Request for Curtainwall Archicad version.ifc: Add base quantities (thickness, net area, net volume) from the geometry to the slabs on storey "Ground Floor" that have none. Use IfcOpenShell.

First a look at what the model holds.

```python
import ifcopenshell
import ifcopenshell.util.element
import ifcopenshell.util.unit

model = ifcopenshell.open("Curtainwall Archicad version.ifc")
print(model.schema)
for unit_type in ("LENGTHUNIT", "AREAUNIT", "VOLUMEUNIT"):
    print(unit_type, ifcopenshell.util.unit.calculate_unit_scale(model, unit_type))
storey = next(s for s in model.by_type("IfcBuildingStorey") if s.Name == "Ground Floor")
slabs = [e for e in ifcopenshell.util.element.get_decomposition(storey) if e.is_a("IfcSlab")]
for e in sorted(slabs, key=lambda e: e.id()):
    print(e.id(), e.is_a(), e.Name, list(ifcopenshell.util.element.get_psets(e, qtos_only=True)), sep=" | ")
```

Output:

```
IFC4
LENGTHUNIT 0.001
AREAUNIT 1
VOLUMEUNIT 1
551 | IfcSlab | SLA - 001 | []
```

```python
import ifcopenshell
import ifcopenshell.api.pset
import ifcopenshell.geom
import ifcopenshell.util.element
import ifcopenshell.util.shape
import ifcopenshell.util.unit

model = ifcopenshell.open("Curtainwall Archicad version.ifc")
unit_scale = ifcopenshell.util.unit.calculate_unit_scale(model)
area_scale = ifcopenshell.util.unit.calculate_unit_scale(model, "AREAUNIT")
volume_scale = ifcopenshell.util.unit.calculate_unit_scale(model, "VOLUMEUNIT")
settings = ifcopenshell.geom.settings()

storey = next(s for s in model.by_type("IfcBuildingStorey") if s.Name == "Ground Floor")
slabs = [e for e in ifcopenshell.util.element.get_decomposition(storey) if e.is_a("IfcSlab")]

for e in sorted(slabs, key=lambda e: e.id()):
    if ifcopenshell.util.element.get_psets(e, qtos_only=True, should_inherit=False):
        continue
    # Geometry comes back in metres, in the element's own axes.
    shape = ifcopenshell.geom.create_shape(settings, e)
    values = {
        "Width": ifcopenshell.util.shape.get_z(shape.geometry) / unit_scale,
        "NetArea": ifcopenshell.util.shape.get_footprint_area(shape.geometry) / area_scale,
        "NetVolume": ifcopenshell.util.shape.get_volume(shape.geometry) / volume_scale,
    }
    qto = ifcopenshell.api.pset.add_qto(model, product=e, name="Qto_SlabBaseQuantities")
    ifcopenshell.api.pset.edit_qto(model, qto=qto, properties=values)
    print(e.id(), {k: round(v, 3) for k, v in values.items()})

model.write("Curtainwall Archicad version_updated.ifc")
```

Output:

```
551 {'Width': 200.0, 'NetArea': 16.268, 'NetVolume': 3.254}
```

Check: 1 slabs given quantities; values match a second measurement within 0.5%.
